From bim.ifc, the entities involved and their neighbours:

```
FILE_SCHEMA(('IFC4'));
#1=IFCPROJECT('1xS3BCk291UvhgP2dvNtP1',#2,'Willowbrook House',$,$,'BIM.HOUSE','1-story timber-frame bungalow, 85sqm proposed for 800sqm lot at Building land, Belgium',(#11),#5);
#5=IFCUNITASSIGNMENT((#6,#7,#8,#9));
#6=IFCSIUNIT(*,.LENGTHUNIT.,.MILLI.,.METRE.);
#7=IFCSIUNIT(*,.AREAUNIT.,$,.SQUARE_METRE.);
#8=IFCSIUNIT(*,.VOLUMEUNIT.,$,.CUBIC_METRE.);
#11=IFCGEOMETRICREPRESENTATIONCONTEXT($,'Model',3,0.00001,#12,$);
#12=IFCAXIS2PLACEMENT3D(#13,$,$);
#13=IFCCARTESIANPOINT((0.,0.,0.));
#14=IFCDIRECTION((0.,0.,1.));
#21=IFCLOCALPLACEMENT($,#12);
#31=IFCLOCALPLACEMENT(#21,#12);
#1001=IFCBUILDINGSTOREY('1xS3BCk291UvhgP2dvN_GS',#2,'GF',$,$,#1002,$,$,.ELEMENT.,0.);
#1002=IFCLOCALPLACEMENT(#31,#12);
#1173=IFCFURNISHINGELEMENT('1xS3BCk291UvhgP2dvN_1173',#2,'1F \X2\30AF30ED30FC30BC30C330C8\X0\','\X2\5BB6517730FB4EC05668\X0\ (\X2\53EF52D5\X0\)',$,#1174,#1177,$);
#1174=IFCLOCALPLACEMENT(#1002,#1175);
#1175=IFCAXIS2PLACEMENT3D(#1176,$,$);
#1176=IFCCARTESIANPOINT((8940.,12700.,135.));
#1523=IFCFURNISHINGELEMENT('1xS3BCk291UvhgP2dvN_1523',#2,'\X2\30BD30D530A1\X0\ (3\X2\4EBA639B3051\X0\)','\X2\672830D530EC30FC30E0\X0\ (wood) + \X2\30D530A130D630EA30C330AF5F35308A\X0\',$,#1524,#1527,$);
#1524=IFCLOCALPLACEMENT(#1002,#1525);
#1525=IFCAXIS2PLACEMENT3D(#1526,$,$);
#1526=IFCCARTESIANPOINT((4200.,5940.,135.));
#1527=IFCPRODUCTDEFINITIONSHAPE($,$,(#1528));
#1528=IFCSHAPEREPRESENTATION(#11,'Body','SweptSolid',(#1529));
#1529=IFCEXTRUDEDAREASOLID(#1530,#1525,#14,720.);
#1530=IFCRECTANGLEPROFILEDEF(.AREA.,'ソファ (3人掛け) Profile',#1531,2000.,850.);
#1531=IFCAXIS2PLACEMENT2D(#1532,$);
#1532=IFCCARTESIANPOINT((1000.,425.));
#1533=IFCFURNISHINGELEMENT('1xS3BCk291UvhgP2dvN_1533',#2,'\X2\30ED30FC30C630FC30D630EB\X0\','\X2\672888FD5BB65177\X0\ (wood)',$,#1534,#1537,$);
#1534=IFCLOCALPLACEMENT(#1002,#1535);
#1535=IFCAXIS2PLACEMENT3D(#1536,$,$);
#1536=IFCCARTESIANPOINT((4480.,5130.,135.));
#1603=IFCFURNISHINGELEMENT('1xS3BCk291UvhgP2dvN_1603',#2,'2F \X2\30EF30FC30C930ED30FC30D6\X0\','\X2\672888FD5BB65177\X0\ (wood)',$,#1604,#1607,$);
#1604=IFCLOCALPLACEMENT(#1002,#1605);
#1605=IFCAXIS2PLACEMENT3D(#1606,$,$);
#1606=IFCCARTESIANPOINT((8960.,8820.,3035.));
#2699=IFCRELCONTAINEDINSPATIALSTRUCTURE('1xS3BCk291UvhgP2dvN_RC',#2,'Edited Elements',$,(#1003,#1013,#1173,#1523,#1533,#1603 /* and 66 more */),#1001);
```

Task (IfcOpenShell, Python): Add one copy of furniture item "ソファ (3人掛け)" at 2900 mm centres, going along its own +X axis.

```python
import ifcopenshell
import ifcopenshell.api.geometry
import ifcopenshell.api.root
import ifcopenshell.util.element
import ifcopenshell.util.placement

model = ifcopenshell.open("bim.ifc")


def reuse_history(source, copy):
    """copy_class also copies each property set's owner history, people and application; keep the originals."""
    for rel in copy.IsDefinedBy:
        if rel.is_a("IfcRelDefinesByProperties") and (history := rel.RelatingPropertyDefinition.OwnerHistory):
            rel.RelatingPropertyDefinition.OwnerHistory = source.OwnerHistory
            ifcopenshell.util.element.remove_deep2(model, history)


source = model.by_guid("1xS3BCk291UvhgP2dvN_1523")
base = ifcopenshell.util.placement.get_local_placement(source.ObjectPlacement)
step = base[:3, 0] * 2900.0

for i in range(1, 2):
    copy = ifcopenshell.api.root.copy_class(model, product=source)
    copy.Representation = ifcopenshell.util.element.copy_deep(
        model, source.Representation, exclude=["IfcGeometricRepresentationContext", "IfcRepresentationMap"]
    )
    reuse_history(source, copy)
    matrix = base.copy()
    matrix[:3, 3] += i * step
    print("added at", matrix[:3, 3].round(3) + 0.0)
    ifcopenshell.api.geometry.edit_object_placement(model, product=copy, matrix=matrix, is_si=False)

model.write("bim_rev.ifc")
```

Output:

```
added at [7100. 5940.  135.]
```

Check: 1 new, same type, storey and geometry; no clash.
